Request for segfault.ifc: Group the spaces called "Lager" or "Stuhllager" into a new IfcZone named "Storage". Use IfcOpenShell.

First a look at what the model holds.

```python
import ifcopenshell

model = ifcopenshell.open("segfault.ifc")
print(model.schema)
seen = {}
for space in model.by_type("IfcSpace"):
    seen[space.LongName] = seen.get(space.LongName, 0) + 1
for name, count in sorted(seen.items(), key=str):
    print(count, "x", name)
print("zones:", [z.Name for z in model.by_type("IfcZone")][:20])
```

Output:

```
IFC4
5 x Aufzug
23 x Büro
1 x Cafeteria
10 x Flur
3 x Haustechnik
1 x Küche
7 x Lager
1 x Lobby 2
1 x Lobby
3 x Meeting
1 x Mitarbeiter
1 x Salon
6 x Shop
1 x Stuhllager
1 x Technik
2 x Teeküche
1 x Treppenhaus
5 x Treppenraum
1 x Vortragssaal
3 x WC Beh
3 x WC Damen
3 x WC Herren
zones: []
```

```python
import ifcopenshell
import ifcopenshell.api.group
import ifcopenshell.api.root

model = ifcopenshell.open("segfault.ifc")

names = {"Lager", "Stuhllager"}
spaces = [s for s in model.by_type("IfcSpace") if s.LongName in names]

zone = ifcopenshell.api.root.create_entity(model, ifc_class="IfcZone", name="Storage")
ifcopenshell.api.group.assign_group(model, products=spaces, group=zone)
print(len(spaces), "spaces in", zone.Name)

model.write("segfault_edited.ifc")
```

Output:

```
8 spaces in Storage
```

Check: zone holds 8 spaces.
